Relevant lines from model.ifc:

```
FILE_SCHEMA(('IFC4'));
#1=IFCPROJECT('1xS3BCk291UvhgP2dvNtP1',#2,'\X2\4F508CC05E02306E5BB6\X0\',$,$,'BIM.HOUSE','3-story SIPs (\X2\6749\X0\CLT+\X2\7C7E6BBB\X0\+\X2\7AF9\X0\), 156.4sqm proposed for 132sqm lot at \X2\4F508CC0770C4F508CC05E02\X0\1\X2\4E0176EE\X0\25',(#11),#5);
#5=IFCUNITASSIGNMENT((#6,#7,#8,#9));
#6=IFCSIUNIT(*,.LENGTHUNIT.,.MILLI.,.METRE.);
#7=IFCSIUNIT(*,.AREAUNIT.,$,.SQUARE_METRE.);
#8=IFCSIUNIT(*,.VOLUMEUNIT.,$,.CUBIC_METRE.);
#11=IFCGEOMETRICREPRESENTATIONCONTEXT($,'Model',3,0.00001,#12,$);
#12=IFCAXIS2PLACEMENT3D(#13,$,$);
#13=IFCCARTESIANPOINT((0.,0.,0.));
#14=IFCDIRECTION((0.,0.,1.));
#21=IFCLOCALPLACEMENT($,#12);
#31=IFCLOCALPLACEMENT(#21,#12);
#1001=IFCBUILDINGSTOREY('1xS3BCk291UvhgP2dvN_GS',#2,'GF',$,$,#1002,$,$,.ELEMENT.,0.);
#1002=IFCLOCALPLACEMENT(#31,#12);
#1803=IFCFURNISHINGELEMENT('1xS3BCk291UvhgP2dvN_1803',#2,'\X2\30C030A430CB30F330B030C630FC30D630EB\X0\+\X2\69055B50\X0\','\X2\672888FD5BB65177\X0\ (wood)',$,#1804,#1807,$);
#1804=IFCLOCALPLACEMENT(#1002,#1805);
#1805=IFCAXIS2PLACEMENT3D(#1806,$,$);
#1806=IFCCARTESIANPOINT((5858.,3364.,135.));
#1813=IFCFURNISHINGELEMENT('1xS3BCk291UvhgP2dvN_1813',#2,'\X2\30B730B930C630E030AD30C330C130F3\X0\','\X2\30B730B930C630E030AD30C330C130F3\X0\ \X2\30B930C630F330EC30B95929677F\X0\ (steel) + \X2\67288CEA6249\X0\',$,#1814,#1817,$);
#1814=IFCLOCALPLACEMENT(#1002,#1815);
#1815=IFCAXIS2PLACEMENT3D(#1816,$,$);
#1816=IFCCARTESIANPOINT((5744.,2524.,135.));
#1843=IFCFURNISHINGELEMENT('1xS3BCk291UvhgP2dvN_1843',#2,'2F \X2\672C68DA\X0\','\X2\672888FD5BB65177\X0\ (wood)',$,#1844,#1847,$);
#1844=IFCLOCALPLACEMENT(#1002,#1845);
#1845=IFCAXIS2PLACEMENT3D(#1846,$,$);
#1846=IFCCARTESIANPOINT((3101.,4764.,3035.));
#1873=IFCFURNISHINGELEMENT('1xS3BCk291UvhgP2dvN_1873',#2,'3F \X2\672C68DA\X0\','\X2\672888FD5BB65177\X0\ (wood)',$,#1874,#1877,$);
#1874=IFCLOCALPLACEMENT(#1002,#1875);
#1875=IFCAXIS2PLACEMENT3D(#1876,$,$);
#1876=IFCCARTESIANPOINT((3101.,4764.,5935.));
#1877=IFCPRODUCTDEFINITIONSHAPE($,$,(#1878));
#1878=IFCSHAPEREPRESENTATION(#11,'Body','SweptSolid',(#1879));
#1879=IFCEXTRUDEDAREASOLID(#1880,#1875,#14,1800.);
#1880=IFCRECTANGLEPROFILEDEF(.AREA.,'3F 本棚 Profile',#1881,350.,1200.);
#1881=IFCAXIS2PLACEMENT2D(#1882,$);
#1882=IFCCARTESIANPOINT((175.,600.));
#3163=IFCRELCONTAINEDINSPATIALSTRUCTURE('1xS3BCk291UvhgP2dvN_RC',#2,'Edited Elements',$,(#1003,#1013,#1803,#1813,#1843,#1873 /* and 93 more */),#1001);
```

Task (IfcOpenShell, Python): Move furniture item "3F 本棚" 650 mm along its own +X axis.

```python
import ifcopenshell
import ifcopenshell.api.geometry
import ifcopenshell.util.placement
import ifcopenshell.util.unit

model = ifcopenshell.open("model.ifc")
unit_scale = ifcopenshell.util.unit.calculate_unit_scale(model)

item = model.by_guid("1xS3BCk291UvhgP2dvN_1873")
matrix = ifcopenshell.util.placement.get_local_placement(item.ObjectPlacement)
matrix[:3, 3] += matrix[:3, 0] * 0.65 / unit_scale
ifcopenshell.api.geometry.edit_object_placement(model, product=item, matrix=matrix, is_si=False)

print(ifcopenshell.util.placement.get_local_placement(item.ObjectPlacement).round(3) + 0.0)

model.write("model_v2.ifc")
```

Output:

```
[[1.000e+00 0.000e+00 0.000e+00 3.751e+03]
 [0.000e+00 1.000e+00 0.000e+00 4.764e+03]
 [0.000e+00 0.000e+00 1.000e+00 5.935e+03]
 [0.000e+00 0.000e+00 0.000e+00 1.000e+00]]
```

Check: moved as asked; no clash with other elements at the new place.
